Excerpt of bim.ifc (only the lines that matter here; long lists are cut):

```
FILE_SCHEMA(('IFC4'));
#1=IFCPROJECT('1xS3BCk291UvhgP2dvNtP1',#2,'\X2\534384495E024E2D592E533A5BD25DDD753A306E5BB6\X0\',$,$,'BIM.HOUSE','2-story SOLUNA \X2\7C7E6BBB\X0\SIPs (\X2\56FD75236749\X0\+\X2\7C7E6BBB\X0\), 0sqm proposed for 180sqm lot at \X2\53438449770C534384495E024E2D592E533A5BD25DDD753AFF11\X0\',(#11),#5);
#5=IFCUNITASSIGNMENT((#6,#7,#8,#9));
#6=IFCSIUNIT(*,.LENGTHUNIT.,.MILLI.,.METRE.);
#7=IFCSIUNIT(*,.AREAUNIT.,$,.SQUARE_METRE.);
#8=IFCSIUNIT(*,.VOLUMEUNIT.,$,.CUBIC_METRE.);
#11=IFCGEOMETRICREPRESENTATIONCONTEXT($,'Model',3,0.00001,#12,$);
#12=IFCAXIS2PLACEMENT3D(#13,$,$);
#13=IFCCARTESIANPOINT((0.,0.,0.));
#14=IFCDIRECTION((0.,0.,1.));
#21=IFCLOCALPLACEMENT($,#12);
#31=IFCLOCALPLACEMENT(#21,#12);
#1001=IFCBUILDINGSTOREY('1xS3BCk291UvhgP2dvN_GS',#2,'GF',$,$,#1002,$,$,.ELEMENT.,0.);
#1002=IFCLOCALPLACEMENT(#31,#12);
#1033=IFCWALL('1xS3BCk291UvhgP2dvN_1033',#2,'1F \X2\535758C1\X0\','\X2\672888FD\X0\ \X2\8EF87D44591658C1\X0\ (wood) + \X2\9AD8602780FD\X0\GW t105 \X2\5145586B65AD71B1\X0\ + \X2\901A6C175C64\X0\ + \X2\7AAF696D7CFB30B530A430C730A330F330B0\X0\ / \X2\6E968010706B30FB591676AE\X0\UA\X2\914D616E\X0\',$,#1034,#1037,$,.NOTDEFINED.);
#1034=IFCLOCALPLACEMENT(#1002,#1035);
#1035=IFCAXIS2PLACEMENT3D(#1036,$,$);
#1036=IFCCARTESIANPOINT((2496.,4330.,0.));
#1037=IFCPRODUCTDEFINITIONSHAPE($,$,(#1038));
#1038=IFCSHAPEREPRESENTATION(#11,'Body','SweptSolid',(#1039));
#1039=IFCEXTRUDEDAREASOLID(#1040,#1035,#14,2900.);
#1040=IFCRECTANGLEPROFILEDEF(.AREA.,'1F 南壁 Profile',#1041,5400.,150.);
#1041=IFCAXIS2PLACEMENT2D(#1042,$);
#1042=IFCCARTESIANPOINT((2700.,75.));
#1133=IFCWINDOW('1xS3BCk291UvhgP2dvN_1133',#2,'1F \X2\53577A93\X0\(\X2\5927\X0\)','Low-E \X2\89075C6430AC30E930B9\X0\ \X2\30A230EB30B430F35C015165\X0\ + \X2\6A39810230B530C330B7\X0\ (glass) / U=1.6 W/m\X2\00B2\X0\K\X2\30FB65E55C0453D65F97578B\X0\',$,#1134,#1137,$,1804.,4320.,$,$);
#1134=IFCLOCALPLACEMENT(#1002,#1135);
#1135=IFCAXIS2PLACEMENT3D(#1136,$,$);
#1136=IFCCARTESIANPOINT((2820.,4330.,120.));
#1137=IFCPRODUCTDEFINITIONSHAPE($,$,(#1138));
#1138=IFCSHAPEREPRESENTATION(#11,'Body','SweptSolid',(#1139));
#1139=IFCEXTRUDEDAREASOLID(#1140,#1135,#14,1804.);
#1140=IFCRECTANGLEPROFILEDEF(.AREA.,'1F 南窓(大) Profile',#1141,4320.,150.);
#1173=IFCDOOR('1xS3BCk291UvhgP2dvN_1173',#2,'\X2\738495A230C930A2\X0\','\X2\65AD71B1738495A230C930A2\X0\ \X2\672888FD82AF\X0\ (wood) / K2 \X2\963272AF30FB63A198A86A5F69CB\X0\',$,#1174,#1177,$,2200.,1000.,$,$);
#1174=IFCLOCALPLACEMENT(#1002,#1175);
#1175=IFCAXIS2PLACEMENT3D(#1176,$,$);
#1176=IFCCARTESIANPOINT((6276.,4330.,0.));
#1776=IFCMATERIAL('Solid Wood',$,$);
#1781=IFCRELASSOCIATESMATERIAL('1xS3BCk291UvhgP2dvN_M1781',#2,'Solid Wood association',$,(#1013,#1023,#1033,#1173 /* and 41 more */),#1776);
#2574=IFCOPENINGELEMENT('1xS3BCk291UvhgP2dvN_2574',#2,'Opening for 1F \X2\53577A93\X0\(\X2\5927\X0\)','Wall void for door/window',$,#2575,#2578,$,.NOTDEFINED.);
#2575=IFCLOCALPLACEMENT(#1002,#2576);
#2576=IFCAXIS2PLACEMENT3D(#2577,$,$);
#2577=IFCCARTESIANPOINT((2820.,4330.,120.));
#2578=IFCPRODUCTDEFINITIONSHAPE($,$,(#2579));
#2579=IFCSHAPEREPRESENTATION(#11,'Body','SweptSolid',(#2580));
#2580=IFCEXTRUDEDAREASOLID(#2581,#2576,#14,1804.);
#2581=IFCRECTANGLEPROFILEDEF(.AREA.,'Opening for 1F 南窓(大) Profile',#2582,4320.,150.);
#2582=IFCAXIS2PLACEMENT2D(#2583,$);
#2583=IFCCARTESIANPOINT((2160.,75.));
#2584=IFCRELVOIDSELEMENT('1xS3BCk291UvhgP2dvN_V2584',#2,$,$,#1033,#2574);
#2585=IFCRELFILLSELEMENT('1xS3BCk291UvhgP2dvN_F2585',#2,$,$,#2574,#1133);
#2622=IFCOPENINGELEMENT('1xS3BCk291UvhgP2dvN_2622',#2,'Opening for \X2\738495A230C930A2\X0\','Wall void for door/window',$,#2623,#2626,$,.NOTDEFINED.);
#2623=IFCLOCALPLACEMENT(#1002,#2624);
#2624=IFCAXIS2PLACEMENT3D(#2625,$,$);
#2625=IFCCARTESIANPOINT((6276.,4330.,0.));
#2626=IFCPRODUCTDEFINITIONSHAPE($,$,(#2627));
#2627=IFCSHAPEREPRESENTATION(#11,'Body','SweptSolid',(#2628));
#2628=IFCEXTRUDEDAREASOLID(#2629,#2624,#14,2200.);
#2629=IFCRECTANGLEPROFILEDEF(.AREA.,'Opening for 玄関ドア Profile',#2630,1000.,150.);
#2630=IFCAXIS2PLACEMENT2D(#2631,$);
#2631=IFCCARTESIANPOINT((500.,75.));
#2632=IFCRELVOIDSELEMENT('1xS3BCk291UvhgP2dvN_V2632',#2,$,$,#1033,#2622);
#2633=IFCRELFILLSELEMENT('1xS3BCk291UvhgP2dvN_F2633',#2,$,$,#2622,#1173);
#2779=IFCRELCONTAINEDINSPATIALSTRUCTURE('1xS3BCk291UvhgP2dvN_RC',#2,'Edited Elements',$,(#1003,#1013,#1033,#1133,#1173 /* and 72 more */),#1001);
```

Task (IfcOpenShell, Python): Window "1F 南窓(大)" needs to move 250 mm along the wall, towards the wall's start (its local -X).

```python
import ifcopenshell
import ifcopenshell.api.geometry
import ifcopenshell.util.placement

model = ifcopenshell.open("bim.ifc")

window = model.by_guid("1xS3BCk291UvhgP2dvN_1133")
opening = window.FillsVoids[0].RelatingOpeningElement
wall = opening.VoidsElements[0].RelatingBuildingElement

wall_matrix = ifcopenshell.util.placement.get_local_placement(wall.ObjectPlacement)
shift = wall_matrix[:3, 0] * -250.0
before = ifcopenshell.util.placement.get_local_placement(window.ObjectPlacement)[:3, 3].copy()

# The window is not placed relative to its opening, so move both.
for product in (opening, window):
    matrix = ifcopenshell.util.placement.get_local_placement(product.ObjectPlacement)
    matrix[:3, 3] += shift
    ifcopenshell.api.geometry.edit_object_placement(model, product=product, matrix=matrix, is_si=False)

after = ifcopenshell.util.placement.get_local_placement(window.ObjectPlacement)[:3, 3]
print("window moved by", (after - before).round(3) + 0.0)

model.write("bim_edited.ifc")
```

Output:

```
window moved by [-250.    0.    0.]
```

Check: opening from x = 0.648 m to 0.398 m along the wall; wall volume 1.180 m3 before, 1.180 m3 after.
